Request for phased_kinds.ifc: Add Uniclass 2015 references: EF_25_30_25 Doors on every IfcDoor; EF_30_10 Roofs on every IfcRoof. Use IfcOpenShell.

First a look at what the model holds.

```python
import ifcopenshell

model = ifcopenshell.open("phased_kinds.ifc")
print(model.schema)
print("classifications:", [c.Name for c in model.by_type("IfcClassification")])
for ifc_class in ("IfcDoor", "IfcRoof", "IfcStair", "IfcWall", "IfcWindow"):
    print(ifc_class, len(model.by_type(ifc_class)))
```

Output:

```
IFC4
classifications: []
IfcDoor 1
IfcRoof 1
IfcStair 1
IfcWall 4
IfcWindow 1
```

```python
import ifcopenshell
import ifcopenshell.api.classification

model = ifcopenshell.open("phased_kinds.ifc")

system = ifcopenshell.api.classification.add_classification(model, classification="Uniclass 2015")

codes = {
    "IfcDoor": ("EF_25_30_25", "Doors"),
    "IfcRoof": ("EF_30_10", "Roofs"),
}
for ifc_class, (code, name) in codes.items():
    products = model.by_type(ifc_class)
    ifcopenshell.api.classification.add_reference(
        model, products=products, classification=system, identification=code, name=name
    )
    print(code, len(products))

model.write("phased_kinds_v2.ifc")
```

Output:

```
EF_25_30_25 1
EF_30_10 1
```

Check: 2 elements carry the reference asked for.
